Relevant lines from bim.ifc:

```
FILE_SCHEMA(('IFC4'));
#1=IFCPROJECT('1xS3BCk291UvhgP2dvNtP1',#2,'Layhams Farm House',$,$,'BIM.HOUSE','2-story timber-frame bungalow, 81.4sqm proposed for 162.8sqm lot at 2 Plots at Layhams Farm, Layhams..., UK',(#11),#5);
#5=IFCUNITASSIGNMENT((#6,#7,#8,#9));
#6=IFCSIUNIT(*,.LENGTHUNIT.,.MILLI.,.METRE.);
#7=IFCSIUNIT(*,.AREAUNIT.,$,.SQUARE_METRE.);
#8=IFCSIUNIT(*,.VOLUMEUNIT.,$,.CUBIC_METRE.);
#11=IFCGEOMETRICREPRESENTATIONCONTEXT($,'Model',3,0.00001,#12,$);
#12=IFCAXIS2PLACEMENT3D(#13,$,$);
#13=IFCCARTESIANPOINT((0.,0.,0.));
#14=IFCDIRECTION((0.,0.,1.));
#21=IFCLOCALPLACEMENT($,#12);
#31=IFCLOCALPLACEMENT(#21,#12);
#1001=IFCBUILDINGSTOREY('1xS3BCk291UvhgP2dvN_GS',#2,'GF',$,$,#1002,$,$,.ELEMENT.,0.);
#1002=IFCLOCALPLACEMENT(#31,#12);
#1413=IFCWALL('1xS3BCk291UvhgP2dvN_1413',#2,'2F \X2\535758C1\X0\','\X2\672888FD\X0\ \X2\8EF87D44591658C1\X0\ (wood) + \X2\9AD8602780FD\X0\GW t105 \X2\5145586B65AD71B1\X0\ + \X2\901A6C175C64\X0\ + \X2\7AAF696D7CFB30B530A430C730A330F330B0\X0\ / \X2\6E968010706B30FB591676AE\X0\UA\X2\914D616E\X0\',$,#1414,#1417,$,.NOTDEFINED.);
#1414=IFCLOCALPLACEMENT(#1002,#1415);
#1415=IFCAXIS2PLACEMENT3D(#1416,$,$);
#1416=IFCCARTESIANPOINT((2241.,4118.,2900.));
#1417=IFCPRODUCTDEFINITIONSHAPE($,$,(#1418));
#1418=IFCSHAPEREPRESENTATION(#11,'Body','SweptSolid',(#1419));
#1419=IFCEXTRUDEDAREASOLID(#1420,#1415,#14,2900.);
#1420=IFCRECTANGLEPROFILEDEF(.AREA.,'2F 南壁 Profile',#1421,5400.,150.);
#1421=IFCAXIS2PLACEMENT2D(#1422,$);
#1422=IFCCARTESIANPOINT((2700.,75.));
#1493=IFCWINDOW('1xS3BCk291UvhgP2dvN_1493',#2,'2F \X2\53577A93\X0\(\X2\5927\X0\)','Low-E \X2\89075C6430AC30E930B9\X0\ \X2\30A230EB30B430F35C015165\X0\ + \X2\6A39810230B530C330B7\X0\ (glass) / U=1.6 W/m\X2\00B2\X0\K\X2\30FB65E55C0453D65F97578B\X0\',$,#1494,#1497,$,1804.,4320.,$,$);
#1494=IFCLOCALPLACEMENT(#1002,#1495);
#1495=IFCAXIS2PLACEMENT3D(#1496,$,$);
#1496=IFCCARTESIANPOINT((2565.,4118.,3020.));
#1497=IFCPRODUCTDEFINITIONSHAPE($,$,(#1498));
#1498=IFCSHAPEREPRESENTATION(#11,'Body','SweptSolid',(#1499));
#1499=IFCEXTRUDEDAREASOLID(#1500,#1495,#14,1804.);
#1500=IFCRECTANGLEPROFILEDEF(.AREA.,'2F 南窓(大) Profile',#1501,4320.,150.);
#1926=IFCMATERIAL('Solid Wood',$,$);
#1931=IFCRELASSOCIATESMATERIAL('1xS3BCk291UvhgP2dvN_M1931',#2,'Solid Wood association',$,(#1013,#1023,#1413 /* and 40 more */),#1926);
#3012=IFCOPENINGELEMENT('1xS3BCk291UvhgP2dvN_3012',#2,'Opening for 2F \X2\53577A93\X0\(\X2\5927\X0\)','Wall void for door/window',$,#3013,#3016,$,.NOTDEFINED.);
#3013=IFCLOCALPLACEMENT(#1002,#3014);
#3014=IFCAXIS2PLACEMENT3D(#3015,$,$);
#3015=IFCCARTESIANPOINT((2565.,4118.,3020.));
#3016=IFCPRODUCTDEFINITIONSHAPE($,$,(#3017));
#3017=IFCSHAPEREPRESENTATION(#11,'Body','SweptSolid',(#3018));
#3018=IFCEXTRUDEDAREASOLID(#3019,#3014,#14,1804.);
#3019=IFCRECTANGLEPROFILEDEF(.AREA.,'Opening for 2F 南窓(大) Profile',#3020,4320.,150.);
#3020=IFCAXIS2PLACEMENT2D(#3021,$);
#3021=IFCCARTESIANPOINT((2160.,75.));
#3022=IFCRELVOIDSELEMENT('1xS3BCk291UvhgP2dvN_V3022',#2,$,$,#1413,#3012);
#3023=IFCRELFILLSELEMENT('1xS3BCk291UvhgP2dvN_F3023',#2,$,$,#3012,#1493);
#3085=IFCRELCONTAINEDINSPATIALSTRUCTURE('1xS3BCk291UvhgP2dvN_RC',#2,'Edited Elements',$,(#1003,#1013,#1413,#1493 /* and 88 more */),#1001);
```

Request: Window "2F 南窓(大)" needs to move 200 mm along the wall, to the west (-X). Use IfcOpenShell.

```python
import ifcopenshell
import ifcopenshell.api.geometry
import ifcopenshell.util.placement

model = ifcopenshell.open("bim.ifc")

window = model.by_guid("1xS3BCk291UvhgP2dvN_1493")
opening = window.FillsVoids[0].RelatingOpeningElement
wall = opening.VoidsElements[0].RelatingBuildingElement

wall_matrix = ifcopenshell.util.placement.get_local_placement(wall.ObjectPlacement)
shift = wall_matrix[:3, 0] * -200.0
before = ifcopenshell.util.placement.get_local_placement(window.ObjectPlacement)[:3, 3].copy()

# The window is not placed relative to its opening, so move both.
for product in (opening, window):
    matrix = ifcopenshell.util.placement.get_local_placement(product.ObjectPlacement)
    matrix[:3, 3] += shift
    ifcopenshell.api.geometry.edit_object_placement(model, product=product, matrix=matrix, is_si=False)

after = ifcopenshell.util.placement.get_local_placement(window.ObjectPlacement)[:3, 3]
print("window moved by", (after - before).round(3) + 0.0)

model.write("bim_updated.ifc")
```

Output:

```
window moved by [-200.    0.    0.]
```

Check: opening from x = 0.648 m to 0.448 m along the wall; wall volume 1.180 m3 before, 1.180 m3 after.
